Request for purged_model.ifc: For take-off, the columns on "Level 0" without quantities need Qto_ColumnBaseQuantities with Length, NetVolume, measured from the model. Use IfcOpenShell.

First a look at what the model holds.

```python
import ifcopenshell
import ifcopenshell.util.element
import ifcopenshell.util.unit

model = ifcopenshell.open("purged_model.ifc")
print(model.schema)
for unit_type in ("LENGTHUNIT", "AREAUNIT", "VOLUMEUNIT"):
    print(unit_type, ifcopenshell.util.unit.calculate_unit_scale(model, unit_type))
storey = next(s for s in model.by_type("IfcBuildingStorey") if s.Name == "Level 0")
columns = [e for e in ifcopenshell.util.element.get_decomposition(storey) if e.is_a("IfcColumn")]
for e in sorted(columns, key=lambda e: e.id()):
    print(e.id(), e.is_a(), e.Name, list(ifcopenshell.util.element.get_psets(e, qtos_only=True)), sep=" | ")
```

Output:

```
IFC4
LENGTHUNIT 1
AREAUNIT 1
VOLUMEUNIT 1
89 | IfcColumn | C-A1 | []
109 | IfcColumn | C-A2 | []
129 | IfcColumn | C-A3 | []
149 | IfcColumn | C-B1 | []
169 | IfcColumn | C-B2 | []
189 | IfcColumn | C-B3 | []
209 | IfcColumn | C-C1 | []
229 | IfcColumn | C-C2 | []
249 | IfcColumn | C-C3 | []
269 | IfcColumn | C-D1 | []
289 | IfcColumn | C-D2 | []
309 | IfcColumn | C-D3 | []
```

```python
import ifcopenshell
import ifcopenshell.api.pset
import ifcopenshell.geom
import ifcopenshell.util.element
import ifcopenshell.util.shape
import ifcopenshell.util.unit

model = ifcopenshell.open("purged_model.ifc")
unit_scale = ifcopenshell.util.unit.calculate_unit_scale(model)
volume_scale = ifcopenshell.util.unit.calculate_unit_scale(model, "VOLUMEUNIT")
settings = ifcopenshell.geom.settings()

storey = next(s for s in model.by_type("IfcBuildingStorey") if s.Name == "Level 0")
columns = [e for e in ifcopenshell.util.element.get_decomposition(storey) if e.is_a("IfcColumn")]

for e in sorted(columns, key=lambda e: e.id()):
    if ifcopenshell.util.element.get_psets(e, qtos_only=True, should_inherit=False):
        continue
    # Geometry comes back in metres, in the element's own axes.
    shape = ifcopenshell.geom.create_shape(settings, e)
    values = {
        "Length": ifcopenshell.util.shape.get_z(shape.geometry) / unit_scale,
        "NetVolume": ifcopenshell.util.shape.get_volume(shape.geometry) / volume_scale,
    }
    qto = ifcopenshell.api.pset.add_qto(model, product=e, name="Qto_ColumnBaseQuantities")
    ifcopenshell.api.pset.edit_qto(model, qto=qto, properties=values)
    print(e.id(), {k: round(v, 3) for k, v in values.items()})

model.write("purged_model_updated.ifc")
```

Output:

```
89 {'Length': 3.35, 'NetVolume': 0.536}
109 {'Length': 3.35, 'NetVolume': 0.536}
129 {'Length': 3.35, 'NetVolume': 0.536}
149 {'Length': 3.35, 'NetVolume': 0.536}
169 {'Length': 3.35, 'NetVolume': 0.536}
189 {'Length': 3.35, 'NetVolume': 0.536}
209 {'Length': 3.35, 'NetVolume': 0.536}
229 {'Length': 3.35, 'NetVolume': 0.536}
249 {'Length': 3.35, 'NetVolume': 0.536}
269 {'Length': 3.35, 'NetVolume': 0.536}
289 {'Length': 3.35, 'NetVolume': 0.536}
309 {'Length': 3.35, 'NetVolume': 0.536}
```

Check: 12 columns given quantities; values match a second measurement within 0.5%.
